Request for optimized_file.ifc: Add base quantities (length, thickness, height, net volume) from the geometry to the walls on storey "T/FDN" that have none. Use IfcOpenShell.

First a look at what the model holds.

```python
import ifcopenshell
import ifcopenshell.util.element
import ifcopenshell.util.unit

model = ifcopenshell.open("optimized_file.ifc")
print(model.schema)
for unit_type in ("LENGTHUNIT", "AREAUNIT", "VOLUMEUNIT"):
    print(unit_type, ifcopenshell.util.unit.calculate_unit_scale(model, unit_type))
storey = next(s for s in model.by_type("IfcBuildingStorey") if s.Name == "T/FDN")
walls = [e for e in ifcopenshell.util.element.get_decomposition(storey) if e.is_a("IfcWall")]
for e in sorted(walls, key=lambda e: e.id()):
    print(e.id(), e.is_a(), e.Name, list(ifcopenshell.util.element.get_psets(e, qtos_only=True)), sep=" | ")
```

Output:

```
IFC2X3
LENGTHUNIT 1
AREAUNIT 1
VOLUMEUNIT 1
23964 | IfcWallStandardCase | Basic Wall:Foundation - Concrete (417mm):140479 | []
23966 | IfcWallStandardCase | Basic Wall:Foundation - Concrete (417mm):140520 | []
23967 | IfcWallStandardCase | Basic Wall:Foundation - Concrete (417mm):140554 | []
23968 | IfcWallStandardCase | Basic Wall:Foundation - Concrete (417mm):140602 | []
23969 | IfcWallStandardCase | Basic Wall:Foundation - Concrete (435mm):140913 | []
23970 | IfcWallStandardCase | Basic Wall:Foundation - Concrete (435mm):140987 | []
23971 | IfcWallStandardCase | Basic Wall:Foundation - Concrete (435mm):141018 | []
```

```python
import ifcopenshell
import ifcopenshell.api.pset
import ifcopenshell.geom
import ifcopenshell.util.element
import ifcopenshell.util.shape
import ifcopenshell.util.unit

model = ifcopenshell.open("optimized_file.ifc")
unit_scale = ifcopenshell.util.unit.calculate_unit_scale(model)
volume_scale = ifcopenshell.util.unit.calculate_unit_scale(model, "VOLUMEUNIT")
settings = ifcopenshell.geom.settings()

storey = next(s for s in model.by_type("IfcBuildingStorey") if s.Name == "T/FDN")
walls = [e for e in ifcopenshell.util.element.get_decomposition(storey) if e.is_a("IfcWall")]

for e in sorted(walls, key=lambda e: e.id()):
    if ifcopenshell.util.element.get_psets(e, qtos_only=True, should_inherit=False):
        continue
    # Geometry comes back in metres, in the element's own axes.
    shape = ifcopenshell.geom.create_shape(settings, e)
    values = {
        "Length": ifcopenshell.util.shape.get_x(shape.geometry) / unit_scale,
        "Width": ifcopenshell.util.shape.get_y(shape.geometry) / unit_scale,
        "Height": ifcopenshell.util.shape.get_z(shape.geometry) / unit_scale,
        "NetVolume": ifcopenshell.util.shape.get_volume(shape.geometry) / volume_scale,
    }
    qto = ifcopenshell.api.pset.add_qto(model, product=e, name="BaseQuantities")
    ifcopenshell.api.pset.edit_qto(model, qto=qto, properties=values)
    print(e.id(), {k: round(v, 3) for k, v in values.items()})

model.write("optimized_file_updated.ifc")
```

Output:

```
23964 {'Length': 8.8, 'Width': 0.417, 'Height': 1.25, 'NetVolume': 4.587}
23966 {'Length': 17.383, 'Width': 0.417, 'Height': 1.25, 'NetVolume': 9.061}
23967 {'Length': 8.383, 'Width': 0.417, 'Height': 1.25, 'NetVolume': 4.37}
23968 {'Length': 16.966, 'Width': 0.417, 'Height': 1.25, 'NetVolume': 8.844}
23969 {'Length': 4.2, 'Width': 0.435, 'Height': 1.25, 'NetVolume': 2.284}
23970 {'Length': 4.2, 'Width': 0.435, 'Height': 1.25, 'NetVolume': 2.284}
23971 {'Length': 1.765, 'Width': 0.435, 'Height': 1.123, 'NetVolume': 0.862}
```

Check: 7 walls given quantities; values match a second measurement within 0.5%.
